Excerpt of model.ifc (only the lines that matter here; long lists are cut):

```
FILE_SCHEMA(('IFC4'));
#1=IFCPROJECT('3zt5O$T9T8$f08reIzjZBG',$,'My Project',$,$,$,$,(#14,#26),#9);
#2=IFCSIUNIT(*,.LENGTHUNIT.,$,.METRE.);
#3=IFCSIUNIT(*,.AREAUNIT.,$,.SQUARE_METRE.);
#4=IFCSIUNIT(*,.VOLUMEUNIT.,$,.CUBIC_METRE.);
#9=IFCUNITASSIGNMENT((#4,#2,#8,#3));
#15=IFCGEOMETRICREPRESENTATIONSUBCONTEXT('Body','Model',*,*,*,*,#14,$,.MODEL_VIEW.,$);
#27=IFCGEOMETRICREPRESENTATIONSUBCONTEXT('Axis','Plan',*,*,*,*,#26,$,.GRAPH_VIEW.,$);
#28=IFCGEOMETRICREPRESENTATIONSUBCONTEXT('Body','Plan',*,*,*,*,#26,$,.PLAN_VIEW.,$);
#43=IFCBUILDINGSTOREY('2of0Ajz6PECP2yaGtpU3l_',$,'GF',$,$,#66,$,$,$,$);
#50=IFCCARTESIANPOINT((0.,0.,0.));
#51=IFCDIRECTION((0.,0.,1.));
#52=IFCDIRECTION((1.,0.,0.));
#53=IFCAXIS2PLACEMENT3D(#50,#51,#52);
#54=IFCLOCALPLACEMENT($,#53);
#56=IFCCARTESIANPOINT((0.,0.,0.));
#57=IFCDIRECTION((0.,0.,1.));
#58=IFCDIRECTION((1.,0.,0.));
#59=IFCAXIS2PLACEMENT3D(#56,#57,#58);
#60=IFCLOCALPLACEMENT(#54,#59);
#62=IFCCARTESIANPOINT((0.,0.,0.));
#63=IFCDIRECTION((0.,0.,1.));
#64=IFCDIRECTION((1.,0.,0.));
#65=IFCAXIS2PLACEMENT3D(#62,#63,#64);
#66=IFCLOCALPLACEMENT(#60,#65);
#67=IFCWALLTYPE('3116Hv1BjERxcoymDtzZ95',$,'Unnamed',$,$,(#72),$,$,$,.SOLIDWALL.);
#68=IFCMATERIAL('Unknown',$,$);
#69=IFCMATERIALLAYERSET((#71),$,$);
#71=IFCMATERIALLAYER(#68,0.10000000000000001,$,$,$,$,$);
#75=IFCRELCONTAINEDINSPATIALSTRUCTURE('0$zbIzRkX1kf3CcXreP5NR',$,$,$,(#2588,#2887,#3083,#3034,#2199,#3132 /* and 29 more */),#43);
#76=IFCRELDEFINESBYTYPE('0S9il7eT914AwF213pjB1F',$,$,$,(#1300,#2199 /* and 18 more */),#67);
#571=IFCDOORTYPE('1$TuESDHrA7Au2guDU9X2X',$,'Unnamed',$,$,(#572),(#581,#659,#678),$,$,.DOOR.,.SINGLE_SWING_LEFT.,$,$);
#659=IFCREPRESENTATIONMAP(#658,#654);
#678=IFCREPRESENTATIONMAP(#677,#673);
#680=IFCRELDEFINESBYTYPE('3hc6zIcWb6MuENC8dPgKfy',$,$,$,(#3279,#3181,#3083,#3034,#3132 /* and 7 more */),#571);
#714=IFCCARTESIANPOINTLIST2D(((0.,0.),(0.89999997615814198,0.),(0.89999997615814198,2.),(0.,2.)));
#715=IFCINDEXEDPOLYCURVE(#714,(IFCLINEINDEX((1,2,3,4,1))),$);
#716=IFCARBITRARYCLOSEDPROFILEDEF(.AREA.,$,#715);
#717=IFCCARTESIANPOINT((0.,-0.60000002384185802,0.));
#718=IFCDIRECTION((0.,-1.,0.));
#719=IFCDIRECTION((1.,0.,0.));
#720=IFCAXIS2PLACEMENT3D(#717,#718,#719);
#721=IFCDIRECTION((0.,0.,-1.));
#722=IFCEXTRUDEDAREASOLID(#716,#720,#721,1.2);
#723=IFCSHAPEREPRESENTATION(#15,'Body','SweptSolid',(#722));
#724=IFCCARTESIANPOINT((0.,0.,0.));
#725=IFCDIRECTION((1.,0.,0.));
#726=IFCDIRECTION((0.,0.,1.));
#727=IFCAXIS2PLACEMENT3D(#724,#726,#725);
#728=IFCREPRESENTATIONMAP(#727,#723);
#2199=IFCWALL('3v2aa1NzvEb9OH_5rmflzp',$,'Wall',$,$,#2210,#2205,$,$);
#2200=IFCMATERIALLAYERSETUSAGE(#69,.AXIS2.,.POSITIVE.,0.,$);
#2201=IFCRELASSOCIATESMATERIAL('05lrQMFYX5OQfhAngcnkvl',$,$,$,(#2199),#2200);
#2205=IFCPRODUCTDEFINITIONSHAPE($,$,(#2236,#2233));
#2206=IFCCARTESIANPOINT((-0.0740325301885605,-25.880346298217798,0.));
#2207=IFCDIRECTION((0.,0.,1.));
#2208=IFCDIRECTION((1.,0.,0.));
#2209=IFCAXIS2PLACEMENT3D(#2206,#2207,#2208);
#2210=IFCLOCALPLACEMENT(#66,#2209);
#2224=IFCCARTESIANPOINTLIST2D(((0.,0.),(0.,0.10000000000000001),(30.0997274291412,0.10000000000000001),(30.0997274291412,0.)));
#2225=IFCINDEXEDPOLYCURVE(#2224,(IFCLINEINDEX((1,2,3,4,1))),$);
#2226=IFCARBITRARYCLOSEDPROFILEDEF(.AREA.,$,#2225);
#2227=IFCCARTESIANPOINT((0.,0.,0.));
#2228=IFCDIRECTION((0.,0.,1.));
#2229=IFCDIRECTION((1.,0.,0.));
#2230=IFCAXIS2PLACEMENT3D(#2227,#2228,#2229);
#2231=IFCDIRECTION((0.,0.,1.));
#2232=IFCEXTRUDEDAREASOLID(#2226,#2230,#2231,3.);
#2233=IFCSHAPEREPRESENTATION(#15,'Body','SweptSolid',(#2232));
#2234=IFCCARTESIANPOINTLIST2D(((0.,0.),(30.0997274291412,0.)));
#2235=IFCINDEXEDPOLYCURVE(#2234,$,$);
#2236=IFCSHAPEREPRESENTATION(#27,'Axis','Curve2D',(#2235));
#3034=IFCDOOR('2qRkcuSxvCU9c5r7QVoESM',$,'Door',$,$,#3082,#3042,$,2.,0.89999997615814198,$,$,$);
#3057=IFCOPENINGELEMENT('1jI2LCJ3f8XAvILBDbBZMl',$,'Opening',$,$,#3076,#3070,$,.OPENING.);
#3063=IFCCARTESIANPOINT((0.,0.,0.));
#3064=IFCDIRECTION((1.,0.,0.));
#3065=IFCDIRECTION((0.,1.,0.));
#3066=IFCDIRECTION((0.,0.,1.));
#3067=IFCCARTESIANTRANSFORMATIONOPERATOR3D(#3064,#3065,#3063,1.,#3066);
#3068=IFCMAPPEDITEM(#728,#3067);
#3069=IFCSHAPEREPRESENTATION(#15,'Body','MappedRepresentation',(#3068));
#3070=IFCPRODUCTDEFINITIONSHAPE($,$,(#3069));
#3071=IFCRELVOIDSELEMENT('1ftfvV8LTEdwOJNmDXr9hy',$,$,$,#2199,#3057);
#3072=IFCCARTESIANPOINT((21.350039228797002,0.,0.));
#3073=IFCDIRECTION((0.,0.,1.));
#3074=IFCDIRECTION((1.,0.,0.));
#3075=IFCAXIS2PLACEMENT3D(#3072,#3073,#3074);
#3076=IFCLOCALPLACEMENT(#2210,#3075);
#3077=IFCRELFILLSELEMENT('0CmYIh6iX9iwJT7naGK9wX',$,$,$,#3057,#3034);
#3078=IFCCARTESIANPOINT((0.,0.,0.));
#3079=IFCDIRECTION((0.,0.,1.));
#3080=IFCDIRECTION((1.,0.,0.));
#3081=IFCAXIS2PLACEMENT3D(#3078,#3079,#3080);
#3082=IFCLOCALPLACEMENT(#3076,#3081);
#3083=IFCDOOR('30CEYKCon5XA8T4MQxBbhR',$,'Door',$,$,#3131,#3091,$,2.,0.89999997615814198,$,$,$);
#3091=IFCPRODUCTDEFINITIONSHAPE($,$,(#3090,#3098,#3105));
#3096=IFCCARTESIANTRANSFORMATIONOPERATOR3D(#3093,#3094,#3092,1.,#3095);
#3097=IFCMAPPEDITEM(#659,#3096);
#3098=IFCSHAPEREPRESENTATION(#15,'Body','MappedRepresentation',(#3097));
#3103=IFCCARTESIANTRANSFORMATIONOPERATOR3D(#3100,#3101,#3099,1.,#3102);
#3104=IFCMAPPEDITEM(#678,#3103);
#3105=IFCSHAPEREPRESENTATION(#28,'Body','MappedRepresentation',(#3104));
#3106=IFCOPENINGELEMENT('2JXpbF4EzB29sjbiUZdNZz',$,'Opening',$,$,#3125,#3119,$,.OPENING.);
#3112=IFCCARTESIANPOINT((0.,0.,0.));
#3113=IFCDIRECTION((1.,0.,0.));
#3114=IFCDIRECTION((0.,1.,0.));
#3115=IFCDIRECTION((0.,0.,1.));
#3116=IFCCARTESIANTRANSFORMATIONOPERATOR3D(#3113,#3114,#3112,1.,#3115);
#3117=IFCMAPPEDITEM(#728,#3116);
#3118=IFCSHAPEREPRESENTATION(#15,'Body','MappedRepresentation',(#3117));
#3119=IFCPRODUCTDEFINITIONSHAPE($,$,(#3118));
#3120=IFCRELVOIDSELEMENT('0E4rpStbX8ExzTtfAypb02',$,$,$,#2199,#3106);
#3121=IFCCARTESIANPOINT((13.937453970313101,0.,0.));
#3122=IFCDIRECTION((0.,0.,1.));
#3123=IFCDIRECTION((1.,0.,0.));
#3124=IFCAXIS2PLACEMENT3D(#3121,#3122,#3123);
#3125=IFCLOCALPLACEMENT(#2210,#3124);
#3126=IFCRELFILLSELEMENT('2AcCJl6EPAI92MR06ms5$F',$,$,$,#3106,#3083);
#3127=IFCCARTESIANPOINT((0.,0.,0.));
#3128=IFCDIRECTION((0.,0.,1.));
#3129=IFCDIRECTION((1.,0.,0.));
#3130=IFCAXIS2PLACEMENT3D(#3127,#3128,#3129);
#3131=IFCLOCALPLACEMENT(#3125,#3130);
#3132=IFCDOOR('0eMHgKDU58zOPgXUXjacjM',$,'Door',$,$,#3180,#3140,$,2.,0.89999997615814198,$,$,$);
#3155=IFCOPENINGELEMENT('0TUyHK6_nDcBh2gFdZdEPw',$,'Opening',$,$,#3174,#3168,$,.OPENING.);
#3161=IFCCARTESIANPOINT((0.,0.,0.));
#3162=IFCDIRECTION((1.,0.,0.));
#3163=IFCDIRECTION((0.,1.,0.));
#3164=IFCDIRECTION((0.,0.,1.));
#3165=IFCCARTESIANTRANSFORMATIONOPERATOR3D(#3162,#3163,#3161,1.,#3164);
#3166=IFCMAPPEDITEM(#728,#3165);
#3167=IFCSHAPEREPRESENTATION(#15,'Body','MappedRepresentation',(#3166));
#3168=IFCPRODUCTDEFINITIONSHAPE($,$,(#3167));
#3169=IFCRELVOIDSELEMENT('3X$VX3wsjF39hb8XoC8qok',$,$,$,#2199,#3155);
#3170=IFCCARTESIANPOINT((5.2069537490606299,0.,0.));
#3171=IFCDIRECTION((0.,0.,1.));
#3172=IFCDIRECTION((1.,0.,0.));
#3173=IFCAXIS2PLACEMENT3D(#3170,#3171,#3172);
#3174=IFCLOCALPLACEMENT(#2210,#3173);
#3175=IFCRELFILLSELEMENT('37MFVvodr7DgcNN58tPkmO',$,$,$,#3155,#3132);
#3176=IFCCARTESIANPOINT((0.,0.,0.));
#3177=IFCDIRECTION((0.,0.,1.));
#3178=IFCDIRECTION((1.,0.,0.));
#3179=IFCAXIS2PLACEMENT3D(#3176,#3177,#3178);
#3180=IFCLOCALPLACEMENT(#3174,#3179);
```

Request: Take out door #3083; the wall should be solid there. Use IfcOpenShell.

```python
import ifcopenshell
import ifcopenshell.api.feature
import ifcopenshell.api.root
import ifcopenshell.geom
import ifcopenshell.util.shape

model = ifcopenshell.open("model.ifc")
settings = ifcopenshell.geom.settings()


def volume(element):
    """Net volume in cubic metres, openings subtracted."""
    shape = ifcopenshell.geom.create_shape(settings, element)
    return ifcopenshell.util.shape.get_volume(shape.geometry)


door = model.by_guid("30CEYKCon5XA8T4MQxBbhR")
opening = door.FillsVoids[0].RelatingOpeningElement
wall = opening.VoidsElements[0].RelatingBuildingElement
before = volume(wall)

ifcopenshell.api.root.remove_product(model, product=door)
ifcopenshell.api.feature.remove_feature(model, feature=opening)

after = volume(wall)

print(f"wall volume {before:.3f} -> {after:.3f} m3")

model.write("model_updated.ifc")
```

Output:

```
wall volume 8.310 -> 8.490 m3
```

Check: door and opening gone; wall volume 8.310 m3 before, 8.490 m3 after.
